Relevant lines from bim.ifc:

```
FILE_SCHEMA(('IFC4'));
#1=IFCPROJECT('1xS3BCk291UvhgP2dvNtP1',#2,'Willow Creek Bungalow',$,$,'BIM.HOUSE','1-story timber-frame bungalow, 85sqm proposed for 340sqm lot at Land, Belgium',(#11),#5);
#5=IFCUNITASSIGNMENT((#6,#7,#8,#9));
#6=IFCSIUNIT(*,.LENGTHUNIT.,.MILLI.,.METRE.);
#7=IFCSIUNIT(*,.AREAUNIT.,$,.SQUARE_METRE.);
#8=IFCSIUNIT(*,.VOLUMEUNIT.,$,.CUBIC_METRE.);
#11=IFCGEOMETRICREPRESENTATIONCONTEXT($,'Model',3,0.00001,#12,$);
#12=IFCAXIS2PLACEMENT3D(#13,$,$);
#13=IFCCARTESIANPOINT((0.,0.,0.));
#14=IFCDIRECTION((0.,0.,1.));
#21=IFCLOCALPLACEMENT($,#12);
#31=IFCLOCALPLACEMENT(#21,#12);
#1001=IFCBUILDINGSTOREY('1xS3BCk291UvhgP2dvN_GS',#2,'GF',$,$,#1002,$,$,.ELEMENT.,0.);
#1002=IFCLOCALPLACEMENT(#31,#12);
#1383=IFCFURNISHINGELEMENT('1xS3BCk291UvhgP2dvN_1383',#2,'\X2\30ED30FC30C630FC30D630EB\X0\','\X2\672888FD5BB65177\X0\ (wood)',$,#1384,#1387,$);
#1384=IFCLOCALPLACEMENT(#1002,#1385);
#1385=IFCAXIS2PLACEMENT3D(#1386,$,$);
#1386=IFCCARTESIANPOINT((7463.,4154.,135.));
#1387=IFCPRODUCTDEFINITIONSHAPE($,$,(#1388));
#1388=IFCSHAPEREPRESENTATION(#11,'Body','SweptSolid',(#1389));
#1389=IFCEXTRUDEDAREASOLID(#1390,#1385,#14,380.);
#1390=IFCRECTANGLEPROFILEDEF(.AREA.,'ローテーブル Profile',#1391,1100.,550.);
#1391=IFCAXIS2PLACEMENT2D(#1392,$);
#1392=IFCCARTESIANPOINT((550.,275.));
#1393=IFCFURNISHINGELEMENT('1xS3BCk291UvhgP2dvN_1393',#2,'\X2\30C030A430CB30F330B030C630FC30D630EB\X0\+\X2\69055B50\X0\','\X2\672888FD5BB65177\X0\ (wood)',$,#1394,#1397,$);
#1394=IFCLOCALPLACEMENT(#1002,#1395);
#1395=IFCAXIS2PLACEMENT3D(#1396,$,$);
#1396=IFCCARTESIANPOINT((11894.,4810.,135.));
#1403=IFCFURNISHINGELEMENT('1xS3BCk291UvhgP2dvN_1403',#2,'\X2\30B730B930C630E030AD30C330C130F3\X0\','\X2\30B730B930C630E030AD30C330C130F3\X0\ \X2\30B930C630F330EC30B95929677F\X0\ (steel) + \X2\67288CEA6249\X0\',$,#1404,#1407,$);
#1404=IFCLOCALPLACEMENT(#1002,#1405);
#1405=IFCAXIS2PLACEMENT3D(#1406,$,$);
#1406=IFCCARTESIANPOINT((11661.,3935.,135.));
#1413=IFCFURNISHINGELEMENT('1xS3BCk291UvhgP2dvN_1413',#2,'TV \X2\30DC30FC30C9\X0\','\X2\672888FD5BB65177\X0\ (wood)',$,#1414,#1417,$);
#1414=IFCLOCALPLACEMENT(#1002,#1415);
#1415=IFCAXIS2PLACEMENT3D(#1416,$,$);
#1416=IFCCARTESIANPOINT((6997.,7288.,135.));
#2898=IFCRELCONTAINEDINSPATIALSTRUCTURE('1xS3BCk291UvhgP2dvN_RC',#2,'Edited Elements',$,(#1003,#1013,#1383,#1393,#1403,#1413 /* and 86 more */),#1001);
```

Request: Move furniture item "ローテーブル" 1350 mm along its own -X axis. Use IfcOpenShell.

```python
import ifcopenshell
import ifcopenshell.api.geometry
import ifcopenshell.util.placement
import ifcopenshell.util.unit

model = ifcopenshell.open("bim.ifc")
unit_scale = ifcopenshell.util.unit.calculate_unit_scale(model)

item = model.by_guid("1xS3BCk291UvhgP2dvN_1383")
matrix = ifcopenshell.util.placement.get_local_placement(item.ObjectPlacement)
matrix[:3, 3] -= matrix[:3, 0] * 1.35 / unit_scale
ifcopenshell.api.geometry.edit_object_placement(model, product=item, matrix=matrix, is_si=False)

print(ifcopenshell.util.placement.get_local_placement(item.ObjectPlacement).round(3) + 0.0)

model.write("bim_edited.ifc")
```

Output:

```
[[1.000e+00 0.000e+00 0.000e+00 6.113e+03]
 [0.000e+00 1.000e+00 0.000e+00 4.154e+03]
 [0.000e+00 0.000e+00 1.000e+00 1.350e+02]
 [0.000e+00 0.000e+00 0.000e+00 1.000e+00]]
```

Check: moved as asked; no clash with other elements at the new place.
